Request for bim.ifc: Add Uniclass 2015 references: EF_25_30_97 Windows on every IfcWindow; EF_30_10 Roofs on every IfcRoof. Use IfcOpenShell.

First a look at what the model holds.

```python
import ifcopenshell

model = ifcopenshell.open("bim.ifc")
print(model.schema)
print("classifications:", [c.Name for c in model.by_type("IfcClassification")])
for ifc_class in ("IfcDoor", "IfcRoof", "IfcStair", "IfcWall", "IfcWindow"):
    print(ifc_class, len(model.by_type(ifc_class)))
```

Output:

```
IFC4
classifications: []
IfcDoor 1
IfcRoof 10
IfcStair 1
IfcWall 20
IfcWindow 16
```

```python
import ifcopenshell
import ifcopenshell.api.classification

model = ifcopenshell.open("bim.ifc")

system = ifcopenshell.api.classification.add_classification(model, classification="Uniclass 2015")

codes = {
    "IfcWindow": ("EF_25_30_97", "Windows"),
    "IfcRoof": ("EF_30_10", "Roofs"),
}
for ifc_class, (code, name) in codes.items():
    products = model.by_type(ifc_class)
    ifcopenshell.api.classification.add_reference(
        model, products=products, classification=system, identification=code, name=name
    )
    print(code, len(products))

model.write("bim_v2.ifc")
```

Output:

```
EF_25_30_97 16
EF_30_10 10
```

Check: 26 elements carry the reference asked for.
